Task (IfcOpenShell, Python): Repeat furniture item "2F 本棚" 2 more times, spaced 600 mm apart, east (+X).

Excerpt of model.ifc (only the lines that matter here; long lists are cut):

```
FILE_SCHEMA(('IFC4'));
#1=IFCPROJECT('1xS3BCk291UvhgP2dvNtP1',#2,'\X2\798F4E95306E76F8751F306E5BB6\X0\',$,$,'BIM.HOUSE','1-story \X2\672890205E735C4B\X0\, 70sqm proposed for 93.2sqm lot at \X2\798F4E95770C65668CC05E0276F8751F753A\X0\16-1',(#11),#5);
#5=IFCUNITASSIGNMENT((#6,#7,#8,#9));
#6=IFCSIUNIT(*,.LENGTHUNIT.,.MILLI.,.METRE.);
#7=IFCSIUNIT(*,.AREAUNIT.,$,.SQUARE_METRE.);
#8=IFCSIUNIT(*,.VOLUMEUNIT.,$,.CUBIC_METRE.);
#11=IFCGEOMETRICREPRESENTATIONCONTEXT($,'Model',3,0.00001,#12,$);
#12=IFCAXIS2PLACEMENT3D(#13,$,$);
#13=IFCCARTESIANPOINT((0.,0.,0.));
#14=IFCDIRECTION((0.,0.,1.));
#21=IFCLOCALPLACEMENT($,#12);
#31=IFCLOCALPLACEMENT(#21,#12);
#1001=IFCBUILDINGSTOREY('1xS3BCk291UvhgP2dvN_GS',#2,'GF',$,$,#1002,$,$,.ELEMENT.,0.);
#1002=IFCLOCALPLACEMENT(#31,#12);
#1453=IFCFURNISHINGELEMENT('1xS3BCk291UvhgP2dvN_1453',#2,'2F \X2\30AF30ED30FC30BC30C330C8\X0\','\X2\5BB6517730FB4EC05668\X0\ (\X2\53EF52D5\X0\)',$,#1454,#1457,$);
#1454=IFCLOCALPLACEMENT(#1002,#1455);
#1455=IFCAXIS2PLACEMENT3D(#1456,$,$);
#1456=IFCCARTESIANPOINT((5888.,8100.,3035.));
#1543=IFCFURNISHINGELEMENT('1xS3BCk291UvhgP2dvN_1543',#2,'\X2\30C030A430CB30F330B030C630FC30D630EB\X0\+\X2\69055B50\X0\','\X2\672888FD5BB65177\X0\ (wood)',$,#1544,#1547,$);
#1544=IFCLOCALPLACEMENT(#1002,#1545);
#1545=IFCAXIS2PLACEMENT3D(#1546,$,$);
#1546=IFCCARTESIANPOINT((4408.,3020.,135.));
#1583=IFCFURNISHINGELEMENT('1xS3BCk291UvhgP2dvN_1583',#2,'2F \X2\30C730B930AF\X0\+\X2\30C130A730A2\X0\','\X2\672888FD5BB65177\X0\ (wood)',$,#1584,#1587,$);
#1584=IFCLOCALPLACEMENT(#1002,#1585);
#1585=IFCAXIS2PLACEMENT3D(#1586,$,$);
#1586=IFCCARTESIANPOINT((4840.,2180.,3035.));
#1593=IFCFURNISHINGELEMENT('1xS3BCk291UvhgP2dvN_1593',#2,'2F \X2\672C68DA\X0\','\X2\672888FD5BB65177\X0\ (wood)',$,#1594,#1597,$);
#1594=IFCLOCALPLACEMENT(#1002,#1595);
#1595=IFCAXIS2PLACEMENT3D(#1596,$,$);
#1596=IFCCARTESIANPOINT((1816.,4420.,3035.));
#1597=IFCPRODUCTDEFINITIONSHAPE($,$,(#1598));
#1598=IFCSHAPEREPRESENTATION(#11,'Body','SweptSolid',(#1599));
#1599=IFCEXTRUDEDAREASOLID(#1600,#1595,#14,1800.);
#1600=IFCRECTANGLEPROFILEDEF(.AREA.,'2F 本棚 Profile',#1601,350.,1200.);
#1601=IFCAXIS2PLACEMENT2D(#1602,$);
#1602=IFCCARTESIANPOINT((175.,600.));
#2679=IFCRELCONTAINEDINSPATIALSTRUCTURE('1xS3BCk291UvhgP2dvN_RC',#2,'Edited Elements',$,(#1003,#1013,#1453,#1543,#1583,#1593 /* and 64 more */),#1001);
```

```python
import numpy as np
import ifcopenshell
import ifcopenshell.api.geometry
import ifcopenshell.api.root
import ifcopenshell.util.element
import ifcopenshell.util.placement
import ifcopenshell.util.unit

model = ifcopenshell.open("model.ifc")
unit_scale = ifcopenshell.util.unit.calculate_unit_scale(model)


def reuse_history(source, copy):
    """copy_class also copies each property set's owner history, people and application; keep the originals."""
    for rel in copy.IsDefinedBy:
        if rel.is_a("IfcRelDefinesByProperties") and (history := rel.RelatingPropertyDefinition.OwnerHistory):
            rel.RelatingPropertyDefinition.OwnerHistory = source.OwnerHistory
            ifcopenshell.util.element.remove_deep2(model, history)


source = model.by_guid("1xS3BCk291UvhgP2dvN_1593")
base = ifcopenshell.util.placement.get_local_placement(source.ObjectPlacement)
step = np.array([1.0, 0.0, 0.0]) * 0.6 / unit_scale

for i in range(1, 3):
    copy = ifcopenshell.api.root.copy_class(model, product=source)
    copy.Representation = ifcopenshell.util.element.copy_deep(
        model, source.Representation, exclude=["IfcGeometricRepresentationContext", "IfcRepresentationMap"]
    )
    reuse_history(source, copy)
    matrix = base.copy()
    matrix[:3, 3] += i * step
    print("added at", matrix[:3, 3].round(3) + 0.0)
    ifcopenshell.api.geometry.edit_object_placement(model, product=copy, matrix=matrix, is_si=False)

model.write("model-out.ifc")
```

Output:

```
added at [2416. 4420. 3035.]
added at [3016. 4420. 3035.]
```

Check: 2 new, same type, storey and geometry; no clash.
